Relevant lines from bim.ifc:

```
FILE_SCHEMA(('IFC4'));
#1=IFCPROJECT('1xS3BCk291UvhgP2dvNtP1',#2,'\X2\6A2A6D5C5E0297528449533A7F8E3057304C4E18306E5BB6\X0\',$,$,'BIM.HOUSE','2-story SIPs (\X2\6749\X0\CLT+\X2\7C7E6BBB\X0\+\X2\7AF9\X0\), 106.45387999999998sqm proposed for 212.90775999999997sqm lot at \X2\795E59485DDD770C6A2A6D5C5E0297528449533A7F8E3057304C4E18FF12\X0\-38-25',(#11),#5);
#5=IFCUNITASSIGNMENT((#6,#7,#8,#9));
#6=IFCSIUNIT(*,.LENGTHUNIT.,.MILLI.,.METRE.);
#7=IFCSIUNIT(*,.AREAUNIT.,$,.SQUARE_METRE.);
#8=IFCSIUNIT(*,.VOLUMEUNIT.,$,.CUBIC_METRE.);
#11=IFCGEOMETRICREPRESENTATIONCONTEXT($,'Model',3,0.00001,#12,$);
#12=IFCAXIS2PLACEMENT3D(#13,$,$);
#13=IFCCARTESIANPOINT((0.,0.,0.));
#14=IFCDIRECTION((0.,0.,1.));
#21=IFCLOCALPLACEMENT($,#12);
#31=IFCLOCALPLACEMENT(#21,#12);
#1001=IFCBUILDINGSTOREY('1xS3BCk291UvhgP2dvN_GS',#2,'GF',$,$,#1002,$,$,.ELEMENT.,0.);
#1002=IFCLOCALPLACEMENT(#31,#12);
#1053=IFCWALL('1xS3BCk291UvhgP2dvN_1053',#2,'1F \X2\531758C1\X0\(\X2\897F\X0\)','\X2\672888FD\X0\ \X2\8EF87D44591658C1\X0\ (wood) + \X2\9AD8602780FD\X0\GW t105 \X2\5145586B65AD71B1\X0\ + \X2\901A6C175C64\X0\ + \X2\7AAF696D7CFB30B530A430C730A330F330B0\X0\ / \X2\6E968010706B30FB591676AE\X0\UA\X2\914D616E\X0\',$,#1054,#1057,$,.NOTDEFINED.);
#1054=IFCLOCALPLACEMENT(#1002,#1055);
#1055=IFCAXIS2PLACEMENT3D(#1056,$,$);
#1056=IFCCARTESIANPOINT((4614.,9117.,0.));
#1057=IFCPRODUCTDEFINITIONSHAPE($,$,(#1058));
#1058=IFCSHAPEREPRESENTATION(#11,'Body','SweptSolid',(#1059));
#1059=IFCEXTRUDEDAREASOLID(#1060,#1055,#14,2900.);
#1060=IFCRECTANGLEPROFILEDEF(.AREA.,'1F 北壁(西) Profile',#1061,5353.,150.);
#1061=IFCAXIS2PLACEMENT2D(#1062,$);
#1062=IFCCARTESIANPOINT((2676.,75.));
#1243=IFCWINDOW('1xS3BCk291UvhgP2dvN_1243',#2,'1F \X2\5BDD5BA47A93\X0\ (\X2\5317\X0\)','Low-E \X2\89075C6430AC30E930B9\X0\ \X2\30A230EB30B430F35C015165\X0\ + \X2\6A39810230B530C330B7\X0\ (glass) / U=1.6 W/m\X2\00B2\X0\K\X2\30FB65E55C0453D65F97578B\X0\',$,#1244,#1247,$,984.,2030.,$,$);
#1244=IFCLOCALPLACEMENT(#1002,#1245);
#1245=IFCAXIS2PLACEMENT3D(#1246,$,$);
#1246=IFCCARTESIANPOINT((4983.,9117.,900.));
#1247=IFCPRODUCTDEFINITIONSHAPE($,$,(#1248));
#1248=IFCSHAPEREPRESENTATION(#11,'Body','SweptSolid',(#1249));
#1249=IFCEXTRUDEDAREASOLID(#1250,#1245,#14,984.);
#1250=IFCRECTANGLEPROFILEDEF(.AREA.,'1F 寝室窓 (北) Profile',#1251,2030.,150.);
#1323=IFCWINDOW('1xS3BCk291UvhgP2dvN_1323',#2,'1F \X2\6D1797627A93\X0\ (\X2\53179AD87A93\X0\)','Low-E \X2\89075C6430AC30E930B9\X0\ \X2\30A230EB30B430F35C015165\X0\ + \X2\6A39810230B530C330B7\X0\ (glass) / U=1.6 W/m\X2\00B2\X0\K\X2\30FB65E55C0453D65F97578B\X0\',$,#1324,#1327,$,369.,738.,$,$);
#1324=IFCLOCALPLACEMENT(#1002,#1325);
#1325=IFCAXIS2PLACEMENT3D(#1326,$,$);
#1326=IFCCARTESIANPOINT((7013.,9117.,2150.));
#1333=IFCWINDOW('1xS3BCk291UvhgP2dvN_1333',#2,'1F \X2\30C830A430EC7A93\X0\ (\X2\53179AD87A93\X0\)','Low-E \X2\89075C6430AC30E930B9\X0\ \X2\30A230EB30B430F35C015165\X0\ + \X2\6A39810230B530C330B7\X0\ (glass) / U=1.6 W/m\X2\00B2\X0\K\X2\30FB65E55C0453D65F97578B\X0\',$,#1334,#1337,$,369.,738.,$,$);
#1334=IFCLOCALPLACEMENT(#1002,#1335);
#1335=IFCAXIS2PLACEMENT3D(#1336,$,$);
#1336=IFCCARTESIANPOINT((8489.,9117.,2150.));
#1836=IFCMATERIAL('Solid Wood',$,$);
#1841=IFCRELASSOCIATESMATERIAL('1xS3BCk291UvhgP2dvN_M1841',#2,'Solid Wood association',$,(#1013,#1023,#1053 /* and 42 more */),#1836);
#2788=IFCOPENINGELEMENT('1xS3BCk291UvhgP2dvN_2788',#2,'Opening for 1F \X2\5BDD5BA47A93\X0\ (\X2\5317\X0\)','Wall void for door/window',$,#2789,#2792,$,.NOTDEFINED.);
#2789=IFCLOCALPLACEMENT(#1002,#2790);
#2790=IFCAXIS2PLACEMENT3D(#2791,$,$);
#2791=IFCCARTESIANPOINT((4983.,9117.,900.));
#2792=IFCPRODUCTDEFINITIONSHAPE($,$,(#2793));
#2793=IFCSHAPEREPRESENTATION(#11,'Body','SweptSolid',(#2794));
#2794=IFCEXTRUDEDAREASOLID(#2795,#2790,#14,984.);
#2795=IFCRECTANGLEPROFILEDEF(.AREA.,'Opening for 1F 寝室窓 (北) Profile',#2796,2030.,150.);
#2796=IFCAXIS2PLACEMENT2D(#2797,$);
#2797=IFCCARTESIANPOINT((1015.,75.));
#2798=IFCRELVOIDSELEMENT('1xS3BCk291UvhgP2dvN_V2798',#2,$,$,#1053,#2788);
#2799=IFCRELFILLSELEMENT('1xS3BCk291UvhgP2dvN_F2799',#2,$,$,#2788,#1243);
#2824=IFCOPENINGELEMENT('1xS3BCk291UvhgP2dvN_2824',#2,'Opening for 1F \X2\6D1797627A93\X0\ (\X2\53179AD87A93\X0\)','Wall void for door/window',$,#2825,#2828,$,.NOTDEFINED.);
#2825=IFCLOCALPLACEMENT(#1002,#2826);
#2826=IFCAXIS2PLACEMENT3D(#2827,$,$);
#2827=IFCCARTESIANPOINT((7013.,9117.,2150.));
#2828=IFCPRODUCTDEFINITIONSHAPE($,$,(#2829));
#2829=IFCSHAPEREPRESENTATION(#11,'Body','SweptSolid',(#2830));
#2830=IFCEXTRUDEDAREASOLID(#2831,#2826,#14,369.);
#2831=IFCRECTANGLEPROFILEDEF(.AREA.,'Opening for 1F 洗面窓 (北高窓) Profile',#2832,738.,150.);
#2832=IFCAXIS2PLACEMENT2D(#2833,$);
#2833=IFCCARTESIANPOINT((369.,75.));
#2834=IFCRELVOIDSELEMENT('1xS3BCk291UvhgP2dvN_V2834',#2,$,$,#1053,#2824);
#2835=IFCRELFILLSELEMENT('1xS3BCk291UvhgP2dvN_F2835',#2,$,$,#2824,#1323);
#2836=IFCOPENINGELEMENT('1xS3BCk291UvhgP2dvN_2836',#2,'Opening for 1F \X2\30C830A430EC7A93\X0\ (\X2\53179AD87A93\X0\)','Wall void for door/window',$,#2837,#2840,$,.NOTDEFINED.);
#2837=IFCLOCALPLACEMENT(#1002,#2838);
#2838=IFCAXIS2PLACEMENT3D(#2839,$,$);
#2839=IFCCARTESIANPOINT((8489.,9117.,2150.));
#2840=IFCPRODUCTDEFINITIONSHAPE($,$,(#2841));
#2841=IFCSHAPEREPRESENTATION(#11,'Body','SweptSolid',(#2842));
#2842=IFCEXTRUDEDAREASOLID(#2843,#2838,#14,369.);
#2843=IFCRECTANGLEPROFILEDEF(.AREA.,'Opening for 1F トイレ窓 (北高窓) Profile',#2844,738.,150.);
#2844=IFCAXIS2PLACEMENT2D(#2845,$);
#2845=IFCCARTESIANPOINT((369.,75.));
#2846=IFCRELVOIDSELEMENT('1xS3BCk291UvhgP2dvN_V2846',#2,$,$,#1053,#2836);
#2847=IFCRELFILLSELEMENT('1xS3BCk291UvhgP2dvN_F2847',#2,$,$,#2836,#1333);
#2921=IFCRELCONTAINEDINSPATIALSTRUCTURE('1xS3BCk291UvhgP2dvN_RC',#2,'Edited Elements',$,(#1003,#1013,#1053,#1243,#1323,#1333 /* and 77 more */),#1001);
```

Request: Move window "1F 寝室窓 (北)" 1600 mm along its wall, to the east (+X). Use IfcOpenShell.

```python
import ifcopenshell
import ifcopenshell.api.geometry
import ifcopenshell.util.placement
import ifcopenshell.util.unit

model = ifcopenshell.open("bim.ifc")
unit_scale = ifcopenshell.util.unit.calculate_unit_scale(model)

window = model.by_id(1243)
opening = window.FillsVoids[0].RelatingOpeningElement
wall = opening.VoidsElements[0].RelatingBuildingElement

wall_matrix = ifcopenshell.util.placement.get_local_placement(wall.ObjectPlacement)
shift = wall_matrix[:3, 0] * 1.6 / unit_scale
before = ifcopenshell.util.placement.get_local_placement(window.ObjectPlacement)[:3, 3].copy()

# The window is not placed relative to its opening, so move both.
for product in (opening, window):
    matrix = ifcopenshell.util.placement.get_local_placement(product.ObjectPlacement)
    matrix[:3, 3] += shift
    ifcopenshell.api.geometry.edit_object_placement(model, product=product, matrix=matrix, is_si=False)

after = ifcopenshell.util.placement.get_local_placement(window.ObjectPlacement)[:3, 3]
print("window moved by", (after - before).round(3) + 0.0)

model.write("bim_v2.ifc")
```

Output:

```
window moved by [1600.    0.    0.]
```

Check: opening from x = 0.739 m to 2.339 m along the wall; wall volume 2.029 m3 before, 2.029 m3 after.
